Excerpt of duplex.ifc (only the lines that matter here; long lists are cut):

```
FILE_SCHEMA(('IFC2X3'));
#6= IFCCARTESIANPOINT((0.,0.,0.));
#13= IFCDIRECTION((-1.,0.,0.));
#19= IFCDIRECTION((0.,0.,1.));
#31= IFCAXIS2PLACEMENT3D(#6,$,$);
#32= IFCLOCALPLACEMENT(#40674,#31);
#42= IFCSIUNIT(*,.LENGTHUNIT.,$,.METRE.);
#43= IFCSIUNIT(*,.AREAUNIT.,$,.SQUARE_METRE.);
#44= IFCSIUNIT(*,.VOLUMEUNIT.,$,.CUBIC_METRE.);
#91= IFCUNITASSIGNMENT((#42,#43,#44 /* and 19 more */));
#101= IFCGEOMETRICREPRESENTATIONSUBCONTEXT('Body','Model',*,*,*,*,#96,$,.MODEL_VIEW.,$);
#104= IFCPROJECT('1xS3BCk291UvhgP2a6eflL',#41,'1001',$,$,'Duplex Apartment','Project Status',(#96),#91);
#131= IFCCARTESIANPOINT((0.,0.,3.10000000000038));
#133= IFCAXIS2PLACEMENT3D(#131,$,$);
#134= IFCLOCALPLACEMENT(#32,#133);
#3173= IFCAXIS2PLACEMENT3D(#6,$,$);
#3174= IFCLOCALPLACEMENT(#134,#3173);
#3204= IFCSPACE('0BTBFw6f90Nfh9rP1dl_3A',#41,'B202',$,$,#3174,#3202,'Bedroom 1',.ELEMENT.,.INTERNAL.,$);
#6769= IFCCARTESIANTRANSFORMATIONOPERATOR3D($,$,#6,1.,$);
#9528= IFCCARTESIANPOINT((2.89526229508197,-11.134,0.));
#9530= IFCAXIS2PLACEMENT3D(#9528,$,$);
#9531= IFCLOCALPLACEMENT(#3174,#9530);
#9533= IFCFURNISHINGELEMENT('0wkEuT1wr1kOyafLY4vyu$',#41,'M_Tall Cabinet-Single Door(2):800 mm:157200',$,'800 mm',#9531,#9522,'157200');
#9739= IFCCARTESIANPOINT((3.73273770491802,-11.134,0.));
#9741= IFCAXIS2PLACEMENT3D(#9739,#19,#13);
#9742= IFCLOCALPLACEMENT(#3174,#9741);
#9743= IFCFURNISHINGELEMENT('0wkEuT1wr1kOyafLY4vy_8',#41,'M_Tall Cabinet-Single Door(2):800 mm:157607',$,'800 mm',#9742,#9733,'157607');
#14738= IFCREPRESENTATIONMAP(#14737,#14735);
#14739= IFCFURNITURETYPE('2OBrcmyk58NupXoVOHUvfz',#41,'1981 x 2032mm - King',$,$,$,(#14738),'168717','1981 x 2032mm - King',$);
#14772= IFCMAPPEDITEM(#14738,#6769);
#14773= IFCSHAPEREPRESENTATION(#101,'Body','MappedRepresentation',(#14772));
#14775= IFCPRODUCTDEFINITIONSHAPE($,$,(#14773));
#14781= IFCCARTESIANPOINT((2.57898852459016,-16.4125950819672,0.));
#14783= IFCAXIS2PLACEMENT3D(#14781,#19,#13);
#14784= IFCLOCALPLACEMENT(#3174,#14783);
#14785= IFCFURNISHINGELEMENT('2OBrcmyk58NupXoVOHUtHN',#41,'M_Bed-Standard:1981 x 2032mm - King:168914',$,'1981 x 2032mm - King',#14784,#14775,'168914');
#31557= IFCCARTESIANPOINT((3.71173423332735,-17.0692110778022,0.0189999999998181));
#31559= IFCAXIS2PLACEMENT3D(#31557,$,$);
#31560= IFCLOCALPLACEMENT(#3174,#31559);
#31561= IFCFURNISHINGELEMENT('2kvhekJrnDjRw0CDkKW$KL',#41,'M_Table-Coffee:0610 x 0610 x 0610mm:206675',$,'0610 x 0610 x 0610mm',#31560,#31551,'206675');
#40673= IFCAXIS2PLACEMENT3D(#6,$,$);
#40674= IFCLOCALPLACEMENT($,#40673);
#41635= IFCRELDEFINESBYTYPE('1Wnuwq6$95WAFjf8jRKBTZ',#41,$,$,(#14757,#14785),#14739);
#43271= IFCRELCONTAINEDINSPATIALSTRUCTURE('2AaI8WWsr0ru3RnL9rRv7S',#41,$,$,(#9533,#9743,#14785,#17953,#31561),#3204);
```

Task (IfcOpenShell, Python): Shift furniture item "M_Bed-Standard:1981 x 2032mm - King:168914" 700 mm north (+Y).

```python
import ifcopenshell
import ifcopenshell.api.geometry
import ifcopenshell.util.placement
import ifcopenshell.util.unit

model = ifcopenshell.open("duplex.ifc")
unit_scale = ifcopenshell.util.unit.calculate_unit_scale(model)

item = model.by_id(14785)
matrix = ifcopenshell.util.placement.get_local_placement(item.ObjectPlacement)
matrix[1, 3] += 0.7 / unit_scale
ifcopenshell.api.geometry.edit_object_placement(model, product=item, matrix=matrix, is_si=False)

print(ifcopenshell.util.placement.get_local_placement(item.ObjectPlacement).round(3) + 0.0)

model.write("duplex_v2.ifc")
```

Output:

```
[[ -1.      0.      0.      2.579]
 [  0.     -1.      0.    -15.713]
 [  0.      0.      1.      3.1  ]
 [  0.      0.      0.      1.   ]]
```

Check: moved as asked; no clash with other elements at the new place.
